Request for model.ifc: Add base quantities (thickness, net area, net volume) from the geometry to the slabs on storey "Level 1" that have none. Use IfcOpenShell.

First a look at what the model holds.

```python
import ifcopenshell
import ifcopenshell.util.element
import ifcopenshell.util.unit

model = ifcopenshell.open("model.ifc")
print(model.schema)
for unit_type in ("LENGTHUNIT", "AREAUNIT", "VOLUMEUNIT"):
    print(unit_type, ifcopenshell.util.unit.calculate_unit_scale(model, unit_type))
storey = next(s for s in model.by_type("IfcBuildingStorey") if s.Name == "Level 1")
slabs = [e for e in ifcopenshell.util.element.get_decomposition(storey) if e.is_a("IfcSlab")]
for e in sorted(slabs, key=lambda e: e.id()):
    print(e.id(), e.is_a(), e.Name, list(ifcopenshell.util.element.get_psets(e, qtos_only=True)), sep=" | ")
```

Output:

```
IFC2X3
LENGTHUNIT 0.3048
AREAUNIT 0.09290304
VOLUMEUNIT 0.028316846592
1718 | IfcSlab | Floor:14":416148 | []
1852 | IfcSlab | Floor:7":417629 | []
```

```python
import ifcopenshell
import ifcopenshell.api.pset
import ifcopenshell.geom
import ifcopenshell.util.element
import ifcopenshell.util.shape
import ifcopenshell.util.unit

model = ifcopenshell.open("model.ifc")
unit_scale = ifcopenshell.util.unit.calculate_unit_scale(model)
area_scale = ifcopenshell.util.unit.calculate_unit_scale(model, "AREAUNIT")
volume_scale = ifcopenshell.util.unit.calculate_unit_scale(model, "VOLUMEUNIT")
settings = ifcopenshell.geom.settings()

storey = next(s for s in model.by_type("IfcBuildingStorey") if s.Name == "Level 1")
slabs = [e for e in ifcopenshell.util.element.get_decomposition(storey) if e.is_a("IfcSlab")]

for e in sorted(slabs, key=lambda e: e.id()):
    if ifcopenshell.util.element.get_psets(e, qtos_only=True, should_inherit=False):
        continue
    # Geometry comes back in metres, in the element's own axes.
    shape = ifcopenshell.geom.create_shape(settings, e)
    values = {
        "Width": ifcopenshell.util.shape.get_z(shape.geometry) / unit_scale,
        "NetArea": ifcopenshell.util.shape.get_footprint_area(shape.geometry) / area_scale,
        "NetVolume": ifcopenshell.util.shape.get_volume(shape.geometry) / volume_scale,
    }
    qto = ifcopenshell.api.pset.add_qto(model, product=e, name="BaseQuantities")
    ifcopenshell.api.pset.edit_qto(model, qto=qto, properties=values)
    print(e.id(), {k: round(v, 3) for k, v in values.items()})

model.write("model_rev.ifc")
```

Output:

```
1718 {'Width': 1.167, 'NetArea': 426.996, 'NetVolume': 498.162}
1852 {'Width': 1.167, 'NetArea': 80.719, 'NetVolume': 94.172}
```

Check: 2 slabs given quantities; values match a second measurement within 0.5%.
